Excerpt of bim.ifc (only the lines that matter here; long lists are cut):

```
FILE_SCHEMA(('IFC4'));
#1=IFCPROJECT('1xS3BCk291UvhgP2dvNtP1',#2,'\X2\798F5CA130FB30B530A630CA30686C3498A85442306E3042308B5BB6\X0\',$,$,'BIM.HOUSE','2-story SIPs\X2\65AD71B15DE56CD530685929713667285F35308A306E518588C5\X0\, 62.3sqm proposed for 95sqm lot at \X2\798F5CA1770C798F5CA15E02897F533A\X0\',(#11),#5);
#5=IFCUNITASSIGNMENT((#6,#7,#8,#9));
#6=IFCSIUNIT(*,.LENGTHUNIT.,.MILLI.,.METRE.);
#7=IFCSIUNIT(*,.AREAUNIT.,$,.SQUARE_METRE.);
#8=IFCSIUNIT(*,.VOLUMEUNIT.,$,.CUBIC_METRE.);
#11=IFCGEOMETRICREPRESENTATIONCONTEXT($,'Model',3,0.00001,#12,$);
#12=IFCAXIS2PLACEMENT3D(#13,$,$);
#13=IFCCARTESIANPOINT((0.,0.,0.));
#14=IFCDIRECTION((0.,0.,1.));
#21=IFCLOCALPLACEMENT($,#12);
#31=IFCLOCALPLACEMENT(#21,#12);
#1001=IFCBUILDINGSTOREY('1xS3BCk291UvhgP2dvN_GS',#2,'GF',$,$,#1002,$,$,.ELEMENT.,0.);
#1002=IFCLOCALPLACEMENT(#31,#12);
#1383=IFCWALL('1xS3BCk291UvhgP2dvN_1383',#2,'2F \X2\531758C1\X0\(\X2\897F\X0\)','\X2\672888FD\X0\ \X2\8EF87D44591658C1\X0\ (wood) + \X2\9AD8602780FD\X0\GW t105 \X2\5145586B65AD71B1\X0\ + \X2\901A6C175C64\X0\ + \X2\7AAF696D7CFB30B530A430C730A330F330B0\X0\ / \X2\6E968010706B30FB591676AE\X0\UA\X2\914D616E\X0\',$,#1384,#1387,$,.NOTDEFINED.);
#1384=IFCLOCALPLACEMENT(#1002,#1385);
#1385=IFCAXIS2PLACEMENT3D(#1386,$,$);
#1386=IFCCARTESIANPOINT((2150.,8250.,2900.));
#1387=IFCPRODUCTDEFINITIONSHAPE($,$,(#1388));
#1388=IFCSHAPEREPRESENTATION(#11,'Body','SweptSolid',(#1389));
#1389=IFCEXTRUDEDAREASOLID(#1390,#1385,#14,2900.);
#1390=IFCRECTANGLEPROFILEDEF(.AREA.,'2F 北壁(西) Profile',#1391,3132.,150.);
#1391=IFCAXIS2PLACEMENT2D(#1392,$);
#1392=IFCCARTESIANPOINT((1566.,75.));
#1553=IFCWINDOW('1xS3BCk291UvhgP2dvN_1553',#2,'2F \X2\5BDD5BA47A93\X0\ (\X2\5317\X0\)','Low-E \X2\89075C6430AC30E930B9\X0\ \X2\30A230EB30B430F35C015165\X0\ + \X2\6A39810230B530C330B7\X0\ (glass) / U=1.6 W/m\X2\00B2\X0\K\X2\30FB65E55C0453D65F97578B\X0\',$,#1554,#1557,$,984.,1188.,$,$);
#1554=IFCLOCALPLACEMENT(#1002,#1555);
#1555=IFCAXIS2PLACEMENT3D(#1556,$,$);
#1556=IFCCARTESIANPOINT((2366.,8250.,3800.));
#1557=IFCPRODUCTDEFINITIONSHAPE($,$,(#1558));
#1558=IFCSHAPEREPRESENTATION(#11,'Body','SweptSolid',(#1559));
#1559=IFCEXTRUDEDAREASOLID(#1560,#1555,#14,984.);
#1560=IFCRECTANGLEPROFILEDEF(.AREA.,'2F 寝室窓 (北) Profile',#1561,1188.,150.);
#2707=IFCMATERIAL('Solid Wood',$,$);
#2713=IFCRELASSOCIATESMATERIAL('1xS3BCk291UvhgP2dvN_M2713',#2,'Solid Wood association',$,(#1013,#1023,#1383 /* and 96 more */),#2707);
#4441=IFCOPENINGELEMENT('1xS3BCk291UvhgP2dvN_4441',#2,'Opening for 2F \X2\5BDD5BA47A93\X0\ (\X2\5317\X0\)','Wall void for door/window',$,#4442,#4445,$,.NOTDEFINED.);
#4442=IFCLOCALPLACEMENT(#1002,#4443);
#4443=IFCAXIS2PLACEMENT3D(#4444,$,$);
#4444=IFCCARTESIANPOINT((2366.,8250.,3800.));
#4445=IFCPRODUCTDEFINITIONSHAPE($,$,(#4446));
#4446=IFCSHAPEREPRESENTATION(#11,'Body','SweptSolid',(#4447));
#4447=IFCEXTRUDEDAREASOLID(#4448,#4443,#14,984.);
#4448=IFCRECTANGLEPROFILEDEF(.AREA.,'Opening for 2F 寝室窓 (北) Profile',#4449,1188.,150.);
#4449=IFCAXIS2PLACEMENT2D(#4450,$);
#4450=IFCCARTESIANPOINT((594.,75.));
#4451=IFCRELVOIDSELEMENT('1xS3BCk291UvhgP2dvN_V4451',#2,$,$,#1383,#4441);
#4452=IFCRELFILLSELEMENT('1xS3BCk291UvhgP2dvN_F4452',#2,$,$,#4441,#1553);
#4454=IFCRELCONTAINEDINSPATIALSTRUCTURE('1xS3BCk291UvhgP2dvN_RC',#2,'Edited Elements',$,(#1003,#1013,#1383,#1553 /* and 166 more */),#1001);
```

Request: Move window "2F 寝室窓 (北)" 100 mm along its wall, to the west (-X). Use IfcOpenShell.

```python
import ifcopenshell
import ifcopenshell.api.geometry
import ifcopenshell.util.placement

model = ifcopenshell.open("bim.ifc")

window = model.by_guid("1xS3BCk291UvhgP2dvN_1553")
opening = window.FillsVoids[0].RelatingOpeningElement
wall = opening.VoidsElements[0].RelatingBuildingElement

wall_matrix = ifcopenshell.util.placement.get_local_placement(wall.ObjectPlacement)
shift = wall_matrix[:3, 0] * -100.0
before = ifcopenshell.util.placement.get_local_placement(window.ObjectPlacement)[:3, 3].copy()

# The window is not placed relative to its opening, so move both.
for product in (opening, window):
    matrix = ifcopenshell.util.placement.get_local_placement(product.ObjectPlacement)
    matrix[:3, 3] += shift
    ifcopenshell.api.geometry.edit_object_placement(model, product=product, matrix=matrix, is_si=False)

after = ifcopenshell.util.placement.get_local_placement(window.ObjectPlacement)[:3, 3]
print("window moved by", (after - before).round(3) + 0.0)

model.write("bim_edited.ifc")
```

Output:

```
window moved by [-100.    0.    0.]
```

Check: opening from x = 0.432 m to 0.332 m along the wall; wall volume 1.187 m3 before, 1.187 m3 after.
